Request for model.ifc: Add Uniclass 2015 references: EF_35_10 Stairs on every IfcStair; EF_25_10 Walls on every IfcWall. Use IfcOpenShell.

First a look at what the model holds.

```python
import ifcopenshell

model = ifcopenshell.open("model.ifc")
print(model.schema)
print("classifications:", [c.Name for c in model.by_type("IfcClassification")])
for ifc_class in ("IfcDoor", "IfcRoof", "IfcStair", "IfcWall", "IfcWindow"):
    print(ifc_class, len(model.by_type(ifc_class)))
```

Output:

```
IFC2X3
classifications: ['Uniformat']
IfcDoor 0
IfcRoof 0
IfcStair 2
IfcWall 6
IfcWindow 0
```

```python
import ifcopenshell
import ifcopenshell.api.classification

model = ifcopenshell.open("model.ifc")

# IFC2X3 requires Source and Edition and has no link from the project to the system.
system = model.create_entity("IfcClassification", Source="NBS", Edition="2015", Name="Uniclass 2015")

codes = {
    "IfcStair": ("EF_35_10", "Stairs"),
    "IfcWall": ("EF_25_10", "Walls"),
}
for ifc_class, (code, name) in codes.items():
    products = model.by_type(ifc_class)
    ifcopenshell.api.classification.add_reference(
        model, products=products, classification=system, identification=code, name=name
    )
    print(code, len(products))

model.write("model_rev.ifc")
```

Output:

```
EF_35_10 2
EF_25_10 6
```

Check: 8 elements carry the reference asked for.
